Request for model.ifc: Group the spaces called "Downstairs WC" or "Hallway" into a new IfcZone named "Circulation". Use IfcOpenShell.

First a look at what the model holds.

```python
import ifcopenshell

model = ifcopenshell.open("model.ifc")
print(model.schema)
seen = {}
for space in model.by_type("IfcSpace"):
    seen[space.LongName] = seen.get(space.LongName, 0) + 1
for name, count in sorted(seen.items(), key=str):
    print(count, "x", name)
print("zones:", [z.Name for z in model.by_type("IfcZone")][:20])
```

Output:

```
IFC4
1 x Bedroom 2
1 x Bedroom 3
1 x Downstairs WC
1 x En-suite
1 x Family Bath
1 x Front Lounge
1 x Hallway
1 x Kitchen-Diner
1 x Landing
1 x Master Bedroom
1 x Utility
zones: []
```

```python
import ifcopenshell
import ifcopenshell.api.group
import ifcopenshell.api.root

model = ifcopenshell.open("model.ifc")

names = {"Downstairs WC", "Hallway"}
spaces = [s for s in model.by_type("IfcSpace") if s.LongName in names]

zone = ifcopenshell.api.root.create_entity(model, ifc_class="IfcZone", name="Circulation")
ifcopenshell.api.group.assign_group(model, products=spaces, group=zone)
print(len(spaces), "spaces in", zone.Name)

model.write("model_updated.ifc")
```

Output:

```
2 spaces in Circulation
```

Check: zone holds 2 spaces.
